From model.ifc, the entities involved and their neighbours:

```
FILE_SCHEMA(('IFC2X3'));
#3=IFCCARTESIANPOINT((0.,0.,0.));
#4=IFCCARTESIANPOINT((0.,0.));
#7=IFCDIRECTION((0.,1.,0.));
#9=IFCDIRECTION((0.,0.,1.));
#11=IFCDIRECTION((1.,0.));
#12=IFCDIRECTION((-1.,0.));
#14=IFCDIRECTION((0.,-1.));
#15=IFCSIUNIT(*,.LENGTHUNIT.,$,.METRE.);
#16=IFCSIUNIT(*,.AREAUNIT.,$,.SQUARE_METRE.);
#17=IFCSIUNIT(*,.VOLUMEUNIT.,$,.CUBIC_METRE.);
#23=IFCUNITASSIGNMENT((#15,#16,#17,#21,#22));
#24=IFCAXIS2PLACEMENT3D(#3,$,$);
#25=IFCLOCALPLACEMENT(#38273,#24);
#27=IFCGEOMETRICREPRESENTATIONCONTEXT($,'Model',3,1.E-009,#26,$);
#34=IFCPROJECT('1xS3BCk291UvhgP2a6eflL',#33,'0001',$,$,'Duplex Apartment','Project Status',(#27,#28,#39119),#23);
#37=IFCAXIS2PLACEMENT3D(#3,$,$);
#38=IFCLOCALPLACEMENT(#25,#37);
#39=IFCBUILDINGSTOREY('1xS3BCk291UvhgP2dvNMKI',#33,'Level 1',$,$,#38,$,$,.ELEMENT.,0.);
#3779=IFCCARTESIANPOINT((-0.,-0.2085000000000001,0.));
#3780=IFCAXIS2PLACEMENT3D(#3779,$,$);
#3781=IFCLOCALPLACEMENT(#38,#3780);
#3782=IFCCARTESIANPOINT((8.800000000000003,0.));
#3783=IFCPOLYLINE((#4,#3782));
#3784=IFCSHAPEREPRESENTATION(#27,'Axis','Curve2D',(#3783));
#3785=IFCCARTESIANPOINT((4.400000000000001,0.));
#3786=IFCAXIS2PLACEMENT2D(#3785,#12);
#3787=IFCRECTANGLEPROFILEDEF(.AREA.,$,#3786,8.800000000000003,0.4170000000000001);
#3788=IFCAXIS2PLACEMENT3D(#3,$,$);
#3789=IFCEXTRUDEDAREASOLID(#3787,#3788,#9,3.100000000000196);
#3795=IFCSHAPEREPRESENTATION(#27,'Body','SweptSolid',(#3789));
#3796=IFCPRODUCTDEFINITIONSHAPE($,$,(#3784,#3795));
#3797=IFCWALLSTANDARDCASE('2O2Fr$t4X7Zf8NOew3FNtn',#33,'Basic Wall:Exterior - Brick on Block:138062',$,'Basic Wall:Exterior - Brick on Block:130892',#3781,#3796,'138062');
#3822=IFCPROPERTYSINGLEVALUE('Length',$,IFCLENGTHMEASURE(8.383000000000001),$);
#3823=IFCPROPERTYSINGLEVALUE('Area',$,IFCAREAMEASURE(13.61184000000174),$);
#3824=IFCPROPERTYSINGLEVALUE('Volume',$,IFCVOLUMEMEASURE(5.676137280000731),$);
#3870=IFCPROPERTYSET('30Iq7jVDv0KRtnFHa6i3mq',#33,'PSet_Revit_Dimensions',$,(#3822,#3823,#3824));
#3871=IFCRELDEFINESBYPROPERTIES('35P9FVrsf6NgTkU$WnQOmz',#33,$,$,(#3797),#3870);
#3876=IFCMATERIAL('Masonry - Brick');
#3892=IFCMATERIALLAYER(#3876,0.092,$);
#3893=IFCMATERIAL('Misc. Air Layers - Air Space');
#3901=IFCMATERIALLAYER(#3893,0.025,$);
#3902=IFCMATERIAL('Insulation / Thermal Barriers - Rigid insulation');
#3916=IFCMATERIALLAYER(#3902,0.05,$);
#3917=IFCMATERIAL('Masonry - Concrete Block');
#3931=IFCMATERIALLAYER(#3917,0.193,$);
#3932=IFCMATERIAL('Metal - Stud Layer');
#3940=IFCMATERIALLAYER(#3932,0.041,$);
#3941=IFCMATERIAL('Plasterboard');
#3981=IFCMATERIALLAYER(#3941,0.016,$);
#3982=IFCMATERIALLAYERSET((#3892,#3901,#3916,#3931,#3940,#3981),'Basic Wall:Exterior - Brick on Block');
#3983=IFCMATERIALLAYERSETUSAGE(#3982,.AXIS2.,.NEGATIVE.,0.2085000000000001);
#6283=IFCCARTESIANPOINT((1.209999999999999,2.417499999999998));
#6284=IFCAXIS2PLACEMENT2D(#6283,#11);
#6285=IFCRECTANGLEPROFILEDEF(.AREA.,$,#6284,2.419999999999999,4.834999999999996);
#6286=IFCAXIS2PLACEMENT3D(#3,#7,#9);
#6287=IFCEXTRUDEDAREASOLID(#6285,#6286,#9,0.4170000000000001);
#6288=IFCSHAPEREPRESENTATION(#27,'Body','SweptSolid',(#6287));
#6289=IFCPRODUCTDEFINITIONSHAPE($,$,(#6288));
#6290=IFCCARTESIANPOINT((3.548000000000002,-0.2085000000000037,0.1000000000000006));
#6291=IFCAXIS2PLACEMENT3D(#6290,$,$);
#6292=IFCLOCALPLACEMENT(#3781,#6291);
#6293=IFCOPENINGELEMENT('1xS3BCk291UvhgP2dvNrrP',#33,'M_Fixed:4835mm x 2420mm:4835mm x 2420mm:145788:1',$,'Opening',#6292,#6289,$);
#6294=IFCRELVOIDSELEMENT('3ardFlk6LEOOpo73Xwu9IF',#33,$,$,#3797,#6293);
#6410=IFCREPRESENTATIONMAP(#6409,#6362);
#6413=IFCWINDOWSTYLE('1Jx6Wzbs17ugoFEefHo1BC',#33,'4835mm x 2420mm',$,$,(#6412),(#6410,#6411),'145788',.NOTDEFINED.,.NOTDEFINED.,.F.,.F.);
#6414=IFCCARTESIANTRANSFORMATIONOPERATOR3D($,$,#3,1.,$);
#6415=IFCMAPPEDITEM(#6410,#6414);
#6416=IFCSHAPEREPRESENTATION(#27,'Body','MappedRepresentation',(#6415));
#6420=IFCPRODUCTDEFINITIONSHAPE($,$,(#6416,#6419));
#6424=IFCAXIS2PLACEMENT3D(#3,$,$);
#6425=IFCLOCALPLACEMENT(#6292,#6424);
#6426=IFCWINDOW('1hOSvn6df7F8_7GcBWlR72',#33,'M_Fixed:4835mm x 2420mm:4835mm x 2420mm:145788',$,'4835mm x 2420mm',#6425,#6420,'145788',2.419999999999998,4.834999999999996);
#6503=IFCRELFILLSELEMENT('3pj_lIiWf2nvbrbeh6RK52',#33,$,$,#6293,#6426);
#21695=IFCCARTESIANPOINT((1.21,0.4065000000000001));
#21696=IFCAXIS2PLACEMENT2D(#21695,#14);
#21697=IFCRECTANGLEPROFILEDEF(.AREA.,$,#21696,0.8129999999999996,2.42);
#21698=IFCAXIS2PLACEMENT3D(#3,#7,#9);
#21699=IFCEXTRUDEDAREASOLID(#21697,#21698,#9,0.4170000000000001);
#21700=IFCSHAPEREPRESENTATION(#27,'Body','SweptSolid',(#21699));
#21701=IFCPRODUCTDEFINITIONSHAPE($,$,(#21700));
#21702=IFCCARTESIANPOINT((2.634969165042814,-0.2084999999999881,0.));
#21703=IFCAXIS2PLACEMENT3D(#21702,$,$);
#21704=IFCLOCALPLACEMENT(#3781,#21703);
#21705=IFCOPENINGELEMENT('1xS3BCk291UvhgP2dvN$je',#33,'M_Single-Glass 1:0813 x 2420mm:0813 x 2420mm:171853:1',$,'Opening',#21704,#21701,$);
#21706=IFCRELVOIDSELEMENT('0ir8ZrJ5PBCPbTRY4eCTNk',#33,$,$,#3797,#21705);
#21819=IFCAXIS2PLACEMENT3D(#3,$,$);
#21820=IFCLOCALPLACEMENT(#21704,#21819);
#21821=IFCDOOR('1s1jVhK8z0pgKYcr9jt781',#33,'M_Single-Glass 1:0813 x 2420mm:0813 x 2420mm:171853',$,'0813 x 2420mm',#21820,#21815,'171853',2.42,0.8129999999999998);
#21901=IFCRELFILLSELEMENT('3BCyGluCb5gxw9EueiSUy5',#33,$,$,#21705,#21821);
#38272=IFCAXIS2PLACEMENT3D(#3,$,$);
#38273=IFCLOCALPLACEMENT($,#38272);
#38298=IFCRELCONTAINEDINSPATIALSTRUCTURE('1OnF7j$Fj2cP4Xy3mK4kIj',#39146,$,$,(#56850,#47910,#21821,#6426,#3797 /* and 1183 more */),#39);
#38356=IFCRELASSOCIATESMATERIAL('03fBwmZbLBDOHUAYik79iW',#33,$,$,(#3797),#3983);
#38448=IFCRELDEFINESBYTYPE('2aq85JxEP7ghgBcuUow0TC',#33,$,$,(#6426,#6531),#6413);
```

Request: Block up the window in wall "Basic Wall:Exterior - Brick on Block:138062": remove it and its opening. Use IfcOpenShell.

```python
import ifcopenshell
import ifcopenshell.api.feature
import ifcopenshell.api.pset
import ifcopenshell.api.root
import ifcopenshell.geom
import ifcopenshell.util.element
import ifcopenshell.util.shape
import ifcopenshell.util.unit

model = ifcopenshell.open("model.ifc")
area_scale = ifcopenshell.util.unit.calculate_unit_scale(model, "AREAUNIT")
volume_scale = ifcopenshell.util.unit.calculate_unit_scale(model, "VOLUMEUNIT")
settings = ifcopenshell.geom.settings()


def volume(element):
    """Net volume in cubic metres, openings subtracted."""
    shape = ifcopenshell.geom.create_shape(settings, element)
    return ifcopenshell.util.shape.get_volume(shape.geometry)


window = model.by_id(6426)
opening = window.FillsVoids[0].RelatingOpeningElement
wall = opening.VoidsElements[0].RelatingBuildingElement
before = volume(wall)

ifcopenshell.api.root.remove_product(model, product=window)
ifcopenshell.api.feature.remove_feature(model, feature=opening)

after = volume(wall)
thickness = 0.417  # wall thickness in metres

# Update the wall's stored quantities.
pset = model.by_id(ifcopenshell.util.element.get_pset(wall, "PSet_Revit_Dimensions", should_inherit=False)["id"])
ifcopenshell.api.pset.edit_pset(model, pset=pset, properties={
    "Area": model.create_entity("IfcAreaMeasure", after / thickness / area_scale),
    "Volume": model.create_entity("IfcVolumeMeasure", after / volume_scale),
})

print(f"wall volume {before:.3f} -> {after:.3f} m3")

model.write("model_rev.ifc")
```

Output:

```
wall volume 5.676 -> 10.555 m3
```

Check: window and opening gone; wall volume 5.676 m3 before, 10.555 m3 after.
